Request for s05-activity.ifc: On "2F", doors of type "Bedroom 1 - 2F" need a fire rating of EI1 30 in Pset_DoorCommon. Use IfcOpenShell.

First a look at what the model holds.

```python
import ifcopenshell
import ifcopenshell.util.element

model = ifcopenshell.open("s05-activity.ifc")
print(model.schema)
storey = next(s for s in model.by_type("IfcBuildingStorey") if s.Name == "2F")
doors = [e for e in ifcopenshell.util.element.get_decomposition(storey) if e.is_a("IfcDoor")]
seen = {}
for e in doors:
    element_type = ifcopenshell.util.element.get_type(e)
    key = (element_type.Name if element_type != e and element_type else None, ifcopenshell.util.element.get_pset(e, "Pset_DoorCommon", "FireRating"))
    seen[key] = seen.get(key, 0) + 1
for (name, value), count in sorted(seen.items(), key=str):
    print(count, "x", name, "|", value)
```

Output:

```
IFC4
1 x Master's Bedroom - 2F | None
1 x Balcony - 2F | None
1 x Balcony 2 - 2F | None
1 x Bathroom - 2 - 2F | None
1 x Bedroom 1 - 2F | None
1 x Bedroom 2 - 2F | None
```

```python
import ifcopenshell
import ifcopenshell.api.pset
import ifcopenshell.util.element

model = ifcopenshell.open("s05-activity.ifc")

storey = next(s for s in model.by_type("IfcBuildingStorey") if s.Name == "2F")
doors = [e for e in ifcopenshell.util.element.get_decomposition(storey) if e.is_a("IfcDoor")]

count = 0
for e in doors:
    element_type = ifcopenshell.util.element.get_type(e)
    if element_type in (None, e) or element_type.Name != "Bedroom 1 - 2F":
        continue
    # add_pset returns the element's existing set when there is one.
    pset = ifcopenshell.api.pset.add_pset(model, product=e, name="Pset_DoorCommon")
    ifcopenshell.api.pset.edit_pset(model, pset=pset, properties={"FireRating": "EI1 30"})
    count += 1

print(count, "doors updated")

model.write("s05-activity_updated.ifc")
```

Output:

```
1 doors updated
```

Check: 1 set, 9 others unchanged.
